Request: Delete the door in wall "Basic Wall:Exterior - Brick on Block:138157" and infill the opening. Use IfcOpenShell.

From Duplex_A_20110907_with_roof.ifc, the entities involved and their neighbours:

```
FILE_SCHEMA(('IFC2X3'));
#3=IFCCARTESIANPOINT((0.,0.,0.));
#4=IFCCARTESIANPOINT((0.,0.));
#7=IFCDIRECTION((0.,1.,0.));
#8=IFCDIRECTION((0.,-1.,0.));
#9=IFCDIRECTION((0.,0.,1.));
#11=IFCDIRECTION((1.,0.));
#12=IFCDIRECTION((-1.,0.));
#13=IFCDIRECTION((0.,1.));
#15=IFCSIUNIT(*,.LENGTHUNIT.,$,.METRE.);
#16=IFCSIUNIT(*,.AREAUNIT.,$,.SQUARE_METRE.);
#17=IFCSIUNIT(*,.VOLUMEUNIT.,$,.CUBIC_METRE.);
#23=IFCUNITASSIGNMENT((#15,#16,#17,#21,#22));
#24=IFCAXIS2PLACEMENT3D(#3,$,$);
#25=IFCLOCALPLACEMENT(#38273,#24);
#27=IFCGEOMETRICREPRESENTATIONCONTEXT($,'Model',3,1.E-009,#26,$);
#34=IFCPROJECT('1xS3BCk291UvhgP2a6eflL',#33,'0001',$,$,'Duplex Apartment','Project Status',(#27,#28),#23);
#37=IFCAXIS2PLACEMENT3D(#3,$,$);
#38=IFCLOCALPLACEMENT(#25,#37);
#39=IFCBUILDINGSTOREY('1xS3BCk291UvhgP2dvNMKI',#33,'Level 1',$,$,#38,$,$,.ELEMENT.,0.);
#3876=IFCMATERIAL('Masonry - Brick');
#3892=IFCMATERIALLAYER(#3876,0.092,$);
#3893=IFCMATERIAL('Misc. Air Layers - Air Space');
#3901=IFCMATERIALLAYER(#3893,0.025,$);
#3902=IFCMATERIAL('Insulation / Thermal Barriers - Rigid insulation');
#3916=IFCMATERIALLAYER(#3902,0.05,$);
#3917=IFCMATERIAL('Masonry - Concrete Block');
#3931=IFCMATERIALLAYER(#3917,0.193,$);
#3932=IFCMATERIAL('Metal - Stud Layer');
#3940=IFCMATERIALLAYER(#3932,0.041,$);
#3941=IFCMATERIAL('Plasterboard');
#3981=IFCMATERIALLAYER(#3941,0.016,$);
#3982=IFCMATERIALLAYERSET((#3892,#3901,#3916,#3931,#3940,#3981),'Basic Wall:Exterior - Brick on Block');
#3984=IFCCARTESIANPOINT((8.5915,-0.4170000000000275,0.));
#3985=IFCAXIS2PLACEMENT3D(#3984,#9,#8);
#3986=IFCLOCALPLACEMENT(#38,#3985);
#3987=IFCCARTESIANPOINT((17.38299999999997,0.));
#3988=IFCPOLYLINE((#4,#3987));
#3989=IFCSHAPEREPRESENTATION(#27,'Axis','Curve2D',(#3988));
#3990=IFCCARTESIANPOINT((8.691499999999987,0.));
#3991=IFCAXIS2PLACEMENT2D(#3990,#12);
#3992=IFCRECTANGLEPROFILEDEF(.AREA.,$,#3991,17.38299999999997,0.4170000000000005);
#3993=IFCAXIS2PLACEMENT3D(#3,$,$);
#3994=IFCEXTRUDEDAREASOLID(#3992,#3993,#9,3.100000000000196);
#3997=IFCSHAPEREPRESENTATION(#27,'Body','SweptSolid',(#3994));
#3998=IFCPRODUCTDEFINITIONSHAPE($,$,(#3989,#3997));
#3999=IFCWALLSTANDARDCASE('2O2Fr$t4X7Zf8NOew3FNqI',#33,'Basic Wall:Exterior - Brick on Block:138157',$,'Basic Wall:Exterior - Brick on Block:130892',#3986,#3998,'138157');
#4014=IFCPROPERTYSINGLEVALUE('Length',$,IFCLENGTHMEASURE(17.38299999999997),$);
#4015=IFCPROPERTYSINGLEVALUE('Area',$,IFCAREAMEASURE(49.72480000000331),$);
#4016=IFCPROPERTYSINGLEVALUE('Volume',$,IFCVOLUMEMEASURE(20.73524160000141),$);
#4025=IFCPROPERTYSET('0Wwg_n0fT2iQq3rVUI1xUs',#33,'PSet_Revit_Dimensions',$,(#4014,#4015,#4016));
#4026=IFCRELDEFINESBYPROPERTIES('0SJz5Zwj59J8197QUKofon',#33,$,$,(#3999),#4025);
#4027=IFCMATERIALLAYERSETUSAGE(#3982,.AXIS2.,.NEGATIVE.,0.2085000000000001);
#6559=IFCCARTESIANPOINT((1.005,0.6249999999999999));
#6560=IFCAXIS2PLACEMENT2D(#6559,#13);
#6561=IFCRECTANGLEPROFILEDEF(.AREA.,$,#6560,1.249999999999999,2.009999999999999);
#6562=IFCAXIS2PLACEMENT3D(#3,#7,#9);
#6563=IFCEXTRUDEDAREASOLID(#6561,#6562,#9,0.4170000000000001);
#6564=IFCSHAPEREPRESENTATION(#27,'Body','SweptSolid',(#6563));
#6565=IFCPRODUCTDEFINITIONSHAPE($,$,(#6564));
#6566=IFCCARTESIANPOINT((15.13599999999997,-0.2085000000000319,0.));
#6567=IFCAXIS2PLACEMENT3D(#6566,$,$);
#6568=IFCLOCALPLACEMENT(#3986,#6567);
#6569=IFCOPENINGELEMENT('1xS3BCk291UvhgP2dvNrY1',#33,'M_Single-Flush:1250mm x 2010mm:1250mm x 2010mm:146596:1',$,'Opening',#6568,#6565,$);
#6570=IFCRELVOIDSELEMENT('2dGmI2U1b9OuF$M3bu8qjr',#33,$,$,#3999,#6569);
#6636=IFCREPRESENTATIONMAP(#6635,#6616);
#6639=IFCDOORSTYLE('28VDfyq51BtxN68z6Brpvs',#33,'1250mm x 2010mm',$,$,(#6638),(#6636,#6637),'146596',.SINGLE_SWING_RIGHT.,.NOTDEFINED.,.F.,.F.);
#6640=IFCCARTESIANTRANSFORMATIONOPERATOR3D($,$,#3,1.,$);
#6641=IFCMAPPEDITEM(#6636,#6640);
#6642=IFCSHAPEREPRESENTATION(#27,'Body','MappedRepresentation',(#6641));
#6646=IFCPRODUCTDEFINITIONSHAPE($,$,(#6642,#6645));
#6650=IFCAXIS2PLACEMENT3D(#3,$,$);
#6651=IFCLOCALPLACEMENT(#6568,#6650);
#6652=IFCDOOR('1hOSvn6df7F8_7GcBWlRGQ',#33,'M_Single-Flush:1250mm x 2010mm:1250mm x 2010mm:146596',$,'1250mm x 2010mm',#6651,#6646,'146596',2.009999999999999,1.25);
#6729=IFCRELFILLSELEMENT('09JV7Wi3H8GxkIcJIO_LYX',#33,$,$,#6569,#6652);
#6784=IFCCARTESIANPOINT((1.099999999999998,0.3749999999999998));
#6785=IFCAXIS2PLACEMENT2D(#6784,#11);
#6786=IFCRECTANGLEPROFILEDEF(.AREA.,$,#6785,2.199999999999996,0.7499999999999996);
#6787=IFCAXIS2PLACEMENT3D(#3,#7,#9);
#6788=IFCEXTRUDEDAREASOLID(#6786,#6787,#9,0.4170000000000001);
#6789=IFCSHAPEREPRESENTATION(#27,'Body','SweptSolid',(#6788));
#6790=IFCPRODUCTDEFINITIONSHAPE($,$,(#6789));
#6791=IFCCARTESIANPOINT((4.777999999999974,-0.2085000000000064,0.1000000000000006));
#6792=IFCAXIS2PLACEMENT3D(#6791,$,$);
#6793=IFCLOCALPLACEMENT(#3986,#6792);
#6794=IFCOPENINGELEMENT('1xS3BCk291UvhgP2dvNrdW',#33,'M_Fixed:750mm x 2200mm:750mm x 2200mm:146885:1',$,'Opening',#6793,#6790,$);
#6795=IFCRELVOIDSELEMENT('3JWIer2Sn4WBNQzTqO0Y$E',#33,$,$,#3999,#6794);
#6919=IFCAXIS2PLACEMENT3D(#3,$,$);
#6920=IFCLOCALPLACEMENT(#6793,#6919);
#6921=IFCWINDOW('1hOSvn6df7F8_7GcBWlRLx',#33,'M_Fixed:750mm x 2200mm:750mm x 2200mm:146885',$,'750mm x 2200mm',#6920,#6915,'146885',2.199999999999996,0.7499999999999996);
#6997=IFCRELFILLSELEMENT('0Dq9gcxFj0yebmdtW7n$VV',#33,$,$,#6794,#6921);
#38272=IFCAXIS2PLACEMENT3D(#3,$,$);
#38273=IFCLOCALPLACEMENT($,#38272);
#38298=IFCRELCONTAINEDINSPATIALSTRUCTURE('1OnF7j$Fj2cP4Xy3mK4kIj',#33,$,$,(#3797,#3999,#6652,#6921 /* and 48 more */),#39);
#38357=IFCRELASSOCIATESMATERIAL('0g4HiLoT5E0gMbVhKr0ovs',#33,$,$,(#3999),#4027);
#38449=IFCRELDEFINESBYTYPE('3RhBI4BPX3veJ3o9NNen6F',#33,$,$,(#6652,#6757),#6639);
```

```python
import ifcopenshell
import ifcopenshell.api.feature
import ifcopenshell.api.pset
import ifcopenshell.api.root
import ifcopenshell.geom
import ifcopenshell.util.element
import ifcopenshell.util.shape
import ifcopenshell.util.unit

model = ifcopenshell.open("Duplex_A_20110907_with_roof.ifc")
area_scale = ifcopenshell.util.unit.calculate_unit_scale(model, "AREAUNIT")
volume_scale = ifcopenshell.util.unit.calculate_unit_scale(model, "VOLUMEUNIT")
settings = ifcopenshell.geom.settings()


def volume(element):
    """Net volume in cubic metres, openings subtracted."""
    shape = ifcopenshell.geom.create_shape(settings, element)
    return ifcopenshell.util.shape.get_volume(shape.geometry)


door = model.by_guid("1hOSvn6df7F8_7GcBWlRGQ")
opening = door.FillsVoids[0].RelatingOpeningElement
wall = opening.VoidsElements[0].RelatingBuildingElement
before = volume(wall)

ifcopenshell.api.root.remove_product(model, product=door)
ifcopenshell.api.feature.remove_feature(model, feature=opening)

after = volume(wall)
thickness = 0.417  # wall thickness in metres

# Update the wall's stored quantities.
pset = model.by_id(ifcopenshell.util.element.get_pset(wall, "PSet_Revit_Dimensions", should_inherit=False)["id"])
ifcopenshell.api.pset.edit_pset(model, pset=pset, properties={
    "Area": model.create_entity("IfcAreaMeasure", after / thickness / area_scale),
    "Volume": model.create_entity("IfcVolumeMeasure", after / volume_scale),
})

print(f"wall volume {before:.3f} -> {after:.3f} m3")

model.write("Duplex_A_20110907_with_roof_rev.ifc")
```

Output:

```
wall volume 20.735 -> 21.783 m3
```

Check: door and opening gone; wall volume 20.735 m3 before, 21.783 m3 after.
